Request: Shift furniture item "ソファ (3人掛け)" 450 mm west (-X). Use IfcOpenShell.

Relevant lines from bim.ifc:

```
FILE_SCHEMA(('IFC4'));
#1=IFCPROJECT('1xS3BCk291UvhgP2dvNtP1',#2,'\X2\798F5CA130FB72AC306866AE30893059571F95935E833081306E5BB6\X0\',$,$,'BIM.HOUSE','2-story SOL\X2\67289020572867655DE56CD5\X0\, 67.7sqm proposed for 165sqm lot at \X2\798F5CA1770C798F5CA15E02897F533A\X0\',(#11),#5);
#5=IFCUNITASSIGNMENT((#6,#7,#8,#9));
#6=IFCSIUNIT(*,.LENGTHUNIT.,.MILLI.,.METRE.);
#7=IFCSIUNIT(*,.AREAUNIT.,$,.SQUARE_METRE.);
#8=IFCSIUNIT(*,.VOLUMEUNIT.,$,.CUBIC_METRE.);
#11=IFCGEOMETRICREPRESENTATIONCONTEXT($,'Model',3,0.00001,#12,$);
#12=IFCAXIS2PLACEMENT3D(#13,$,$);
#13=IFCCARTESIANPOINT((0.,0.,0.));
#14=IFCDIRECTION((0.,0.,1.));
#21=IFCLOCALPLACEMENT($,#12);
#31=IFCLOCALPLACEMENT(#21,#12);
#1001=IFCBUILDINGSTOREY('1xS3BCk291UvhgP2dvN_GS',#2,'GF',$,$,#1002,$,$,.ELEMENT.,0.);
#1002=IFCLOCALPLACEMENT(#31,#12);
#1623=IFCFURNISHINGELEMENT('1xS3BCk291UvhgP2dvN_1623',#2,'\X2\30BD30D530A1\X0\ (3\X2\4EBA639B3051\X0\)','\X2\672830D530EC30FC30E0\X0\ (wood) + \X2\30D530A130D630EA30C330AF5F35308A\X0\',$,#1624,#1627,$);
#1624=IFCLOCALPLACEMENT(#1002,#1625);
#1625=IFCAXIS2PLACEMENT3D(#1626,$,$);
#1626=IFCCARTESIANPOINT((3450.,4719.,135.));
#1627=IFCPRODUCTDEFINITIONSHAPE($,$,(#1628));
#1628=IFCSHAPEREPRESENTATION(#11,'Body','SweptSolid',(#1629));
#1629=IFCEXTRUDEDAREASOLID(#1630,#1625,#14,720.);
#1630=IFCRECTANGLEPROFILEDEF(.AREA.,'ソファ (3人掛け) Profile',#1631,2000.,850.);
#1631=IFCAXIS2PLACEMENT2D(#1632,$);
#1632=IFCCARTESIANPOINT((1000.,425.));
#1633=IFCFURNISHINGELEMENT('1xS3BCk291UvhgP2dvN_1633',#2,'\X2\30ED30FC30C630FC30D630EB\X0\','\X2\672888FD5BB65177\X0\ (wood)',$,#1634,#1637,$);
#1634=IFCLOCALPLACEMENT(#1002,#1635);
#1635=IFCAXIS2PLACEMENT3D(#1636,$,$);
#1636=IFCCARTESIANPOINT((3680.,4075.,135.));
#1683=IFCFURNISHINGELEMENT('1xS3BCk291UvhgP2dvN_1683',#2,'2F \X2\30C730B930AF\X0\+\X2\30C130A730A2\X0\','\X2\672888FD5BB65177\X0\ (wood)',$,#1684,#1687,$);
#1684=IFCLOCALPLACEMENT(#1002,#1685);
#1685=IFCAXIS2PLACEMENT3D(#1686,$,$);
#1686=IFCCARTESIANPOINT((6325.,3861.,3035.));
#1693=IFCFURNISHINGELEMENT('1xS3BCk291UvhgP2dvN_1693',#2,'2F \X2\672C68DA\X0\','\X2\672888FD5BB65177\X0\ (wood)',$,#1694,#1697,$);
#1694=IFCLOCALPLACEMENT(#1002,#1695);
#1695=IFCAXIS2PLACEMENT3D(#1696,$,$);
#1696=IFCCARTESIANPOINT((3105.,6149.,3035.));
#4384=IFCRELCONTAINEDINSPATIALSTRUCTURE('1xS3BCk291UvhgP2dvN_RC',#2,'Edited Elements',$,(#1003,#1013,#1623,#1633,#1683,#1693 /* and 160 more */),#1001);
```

```python
import ifcopenshell
import ifcopenshell.api.geometry
import ifcopenshell.util.placement

model = ifcopenshell.open("bim.ifc")

item = model.by_guid("1xS3BCk291UvhgP2dvN_1623")
matrix = ifcopenshell.util.placement.get_local_placement(item.ObjectPlacement)
matrix[0, 3] -= 450.0
ifcopenshell.api.geometry.edit_object_placement(model, product=item, matrix=matrix, is_si=False)

print(ifcopenshell.util.placement.get_local_placement(item.ObjectPlacement).round(3) + 0.0)

model.write("bim_v2.ifc")
```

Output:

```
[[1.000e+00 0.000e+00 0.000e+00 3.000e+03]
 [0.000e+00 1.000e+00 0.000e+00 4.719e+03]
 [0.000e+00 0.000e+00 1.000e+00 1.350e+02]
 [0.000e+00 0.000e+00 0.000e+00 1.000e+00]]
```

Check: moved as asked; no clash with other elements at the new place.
